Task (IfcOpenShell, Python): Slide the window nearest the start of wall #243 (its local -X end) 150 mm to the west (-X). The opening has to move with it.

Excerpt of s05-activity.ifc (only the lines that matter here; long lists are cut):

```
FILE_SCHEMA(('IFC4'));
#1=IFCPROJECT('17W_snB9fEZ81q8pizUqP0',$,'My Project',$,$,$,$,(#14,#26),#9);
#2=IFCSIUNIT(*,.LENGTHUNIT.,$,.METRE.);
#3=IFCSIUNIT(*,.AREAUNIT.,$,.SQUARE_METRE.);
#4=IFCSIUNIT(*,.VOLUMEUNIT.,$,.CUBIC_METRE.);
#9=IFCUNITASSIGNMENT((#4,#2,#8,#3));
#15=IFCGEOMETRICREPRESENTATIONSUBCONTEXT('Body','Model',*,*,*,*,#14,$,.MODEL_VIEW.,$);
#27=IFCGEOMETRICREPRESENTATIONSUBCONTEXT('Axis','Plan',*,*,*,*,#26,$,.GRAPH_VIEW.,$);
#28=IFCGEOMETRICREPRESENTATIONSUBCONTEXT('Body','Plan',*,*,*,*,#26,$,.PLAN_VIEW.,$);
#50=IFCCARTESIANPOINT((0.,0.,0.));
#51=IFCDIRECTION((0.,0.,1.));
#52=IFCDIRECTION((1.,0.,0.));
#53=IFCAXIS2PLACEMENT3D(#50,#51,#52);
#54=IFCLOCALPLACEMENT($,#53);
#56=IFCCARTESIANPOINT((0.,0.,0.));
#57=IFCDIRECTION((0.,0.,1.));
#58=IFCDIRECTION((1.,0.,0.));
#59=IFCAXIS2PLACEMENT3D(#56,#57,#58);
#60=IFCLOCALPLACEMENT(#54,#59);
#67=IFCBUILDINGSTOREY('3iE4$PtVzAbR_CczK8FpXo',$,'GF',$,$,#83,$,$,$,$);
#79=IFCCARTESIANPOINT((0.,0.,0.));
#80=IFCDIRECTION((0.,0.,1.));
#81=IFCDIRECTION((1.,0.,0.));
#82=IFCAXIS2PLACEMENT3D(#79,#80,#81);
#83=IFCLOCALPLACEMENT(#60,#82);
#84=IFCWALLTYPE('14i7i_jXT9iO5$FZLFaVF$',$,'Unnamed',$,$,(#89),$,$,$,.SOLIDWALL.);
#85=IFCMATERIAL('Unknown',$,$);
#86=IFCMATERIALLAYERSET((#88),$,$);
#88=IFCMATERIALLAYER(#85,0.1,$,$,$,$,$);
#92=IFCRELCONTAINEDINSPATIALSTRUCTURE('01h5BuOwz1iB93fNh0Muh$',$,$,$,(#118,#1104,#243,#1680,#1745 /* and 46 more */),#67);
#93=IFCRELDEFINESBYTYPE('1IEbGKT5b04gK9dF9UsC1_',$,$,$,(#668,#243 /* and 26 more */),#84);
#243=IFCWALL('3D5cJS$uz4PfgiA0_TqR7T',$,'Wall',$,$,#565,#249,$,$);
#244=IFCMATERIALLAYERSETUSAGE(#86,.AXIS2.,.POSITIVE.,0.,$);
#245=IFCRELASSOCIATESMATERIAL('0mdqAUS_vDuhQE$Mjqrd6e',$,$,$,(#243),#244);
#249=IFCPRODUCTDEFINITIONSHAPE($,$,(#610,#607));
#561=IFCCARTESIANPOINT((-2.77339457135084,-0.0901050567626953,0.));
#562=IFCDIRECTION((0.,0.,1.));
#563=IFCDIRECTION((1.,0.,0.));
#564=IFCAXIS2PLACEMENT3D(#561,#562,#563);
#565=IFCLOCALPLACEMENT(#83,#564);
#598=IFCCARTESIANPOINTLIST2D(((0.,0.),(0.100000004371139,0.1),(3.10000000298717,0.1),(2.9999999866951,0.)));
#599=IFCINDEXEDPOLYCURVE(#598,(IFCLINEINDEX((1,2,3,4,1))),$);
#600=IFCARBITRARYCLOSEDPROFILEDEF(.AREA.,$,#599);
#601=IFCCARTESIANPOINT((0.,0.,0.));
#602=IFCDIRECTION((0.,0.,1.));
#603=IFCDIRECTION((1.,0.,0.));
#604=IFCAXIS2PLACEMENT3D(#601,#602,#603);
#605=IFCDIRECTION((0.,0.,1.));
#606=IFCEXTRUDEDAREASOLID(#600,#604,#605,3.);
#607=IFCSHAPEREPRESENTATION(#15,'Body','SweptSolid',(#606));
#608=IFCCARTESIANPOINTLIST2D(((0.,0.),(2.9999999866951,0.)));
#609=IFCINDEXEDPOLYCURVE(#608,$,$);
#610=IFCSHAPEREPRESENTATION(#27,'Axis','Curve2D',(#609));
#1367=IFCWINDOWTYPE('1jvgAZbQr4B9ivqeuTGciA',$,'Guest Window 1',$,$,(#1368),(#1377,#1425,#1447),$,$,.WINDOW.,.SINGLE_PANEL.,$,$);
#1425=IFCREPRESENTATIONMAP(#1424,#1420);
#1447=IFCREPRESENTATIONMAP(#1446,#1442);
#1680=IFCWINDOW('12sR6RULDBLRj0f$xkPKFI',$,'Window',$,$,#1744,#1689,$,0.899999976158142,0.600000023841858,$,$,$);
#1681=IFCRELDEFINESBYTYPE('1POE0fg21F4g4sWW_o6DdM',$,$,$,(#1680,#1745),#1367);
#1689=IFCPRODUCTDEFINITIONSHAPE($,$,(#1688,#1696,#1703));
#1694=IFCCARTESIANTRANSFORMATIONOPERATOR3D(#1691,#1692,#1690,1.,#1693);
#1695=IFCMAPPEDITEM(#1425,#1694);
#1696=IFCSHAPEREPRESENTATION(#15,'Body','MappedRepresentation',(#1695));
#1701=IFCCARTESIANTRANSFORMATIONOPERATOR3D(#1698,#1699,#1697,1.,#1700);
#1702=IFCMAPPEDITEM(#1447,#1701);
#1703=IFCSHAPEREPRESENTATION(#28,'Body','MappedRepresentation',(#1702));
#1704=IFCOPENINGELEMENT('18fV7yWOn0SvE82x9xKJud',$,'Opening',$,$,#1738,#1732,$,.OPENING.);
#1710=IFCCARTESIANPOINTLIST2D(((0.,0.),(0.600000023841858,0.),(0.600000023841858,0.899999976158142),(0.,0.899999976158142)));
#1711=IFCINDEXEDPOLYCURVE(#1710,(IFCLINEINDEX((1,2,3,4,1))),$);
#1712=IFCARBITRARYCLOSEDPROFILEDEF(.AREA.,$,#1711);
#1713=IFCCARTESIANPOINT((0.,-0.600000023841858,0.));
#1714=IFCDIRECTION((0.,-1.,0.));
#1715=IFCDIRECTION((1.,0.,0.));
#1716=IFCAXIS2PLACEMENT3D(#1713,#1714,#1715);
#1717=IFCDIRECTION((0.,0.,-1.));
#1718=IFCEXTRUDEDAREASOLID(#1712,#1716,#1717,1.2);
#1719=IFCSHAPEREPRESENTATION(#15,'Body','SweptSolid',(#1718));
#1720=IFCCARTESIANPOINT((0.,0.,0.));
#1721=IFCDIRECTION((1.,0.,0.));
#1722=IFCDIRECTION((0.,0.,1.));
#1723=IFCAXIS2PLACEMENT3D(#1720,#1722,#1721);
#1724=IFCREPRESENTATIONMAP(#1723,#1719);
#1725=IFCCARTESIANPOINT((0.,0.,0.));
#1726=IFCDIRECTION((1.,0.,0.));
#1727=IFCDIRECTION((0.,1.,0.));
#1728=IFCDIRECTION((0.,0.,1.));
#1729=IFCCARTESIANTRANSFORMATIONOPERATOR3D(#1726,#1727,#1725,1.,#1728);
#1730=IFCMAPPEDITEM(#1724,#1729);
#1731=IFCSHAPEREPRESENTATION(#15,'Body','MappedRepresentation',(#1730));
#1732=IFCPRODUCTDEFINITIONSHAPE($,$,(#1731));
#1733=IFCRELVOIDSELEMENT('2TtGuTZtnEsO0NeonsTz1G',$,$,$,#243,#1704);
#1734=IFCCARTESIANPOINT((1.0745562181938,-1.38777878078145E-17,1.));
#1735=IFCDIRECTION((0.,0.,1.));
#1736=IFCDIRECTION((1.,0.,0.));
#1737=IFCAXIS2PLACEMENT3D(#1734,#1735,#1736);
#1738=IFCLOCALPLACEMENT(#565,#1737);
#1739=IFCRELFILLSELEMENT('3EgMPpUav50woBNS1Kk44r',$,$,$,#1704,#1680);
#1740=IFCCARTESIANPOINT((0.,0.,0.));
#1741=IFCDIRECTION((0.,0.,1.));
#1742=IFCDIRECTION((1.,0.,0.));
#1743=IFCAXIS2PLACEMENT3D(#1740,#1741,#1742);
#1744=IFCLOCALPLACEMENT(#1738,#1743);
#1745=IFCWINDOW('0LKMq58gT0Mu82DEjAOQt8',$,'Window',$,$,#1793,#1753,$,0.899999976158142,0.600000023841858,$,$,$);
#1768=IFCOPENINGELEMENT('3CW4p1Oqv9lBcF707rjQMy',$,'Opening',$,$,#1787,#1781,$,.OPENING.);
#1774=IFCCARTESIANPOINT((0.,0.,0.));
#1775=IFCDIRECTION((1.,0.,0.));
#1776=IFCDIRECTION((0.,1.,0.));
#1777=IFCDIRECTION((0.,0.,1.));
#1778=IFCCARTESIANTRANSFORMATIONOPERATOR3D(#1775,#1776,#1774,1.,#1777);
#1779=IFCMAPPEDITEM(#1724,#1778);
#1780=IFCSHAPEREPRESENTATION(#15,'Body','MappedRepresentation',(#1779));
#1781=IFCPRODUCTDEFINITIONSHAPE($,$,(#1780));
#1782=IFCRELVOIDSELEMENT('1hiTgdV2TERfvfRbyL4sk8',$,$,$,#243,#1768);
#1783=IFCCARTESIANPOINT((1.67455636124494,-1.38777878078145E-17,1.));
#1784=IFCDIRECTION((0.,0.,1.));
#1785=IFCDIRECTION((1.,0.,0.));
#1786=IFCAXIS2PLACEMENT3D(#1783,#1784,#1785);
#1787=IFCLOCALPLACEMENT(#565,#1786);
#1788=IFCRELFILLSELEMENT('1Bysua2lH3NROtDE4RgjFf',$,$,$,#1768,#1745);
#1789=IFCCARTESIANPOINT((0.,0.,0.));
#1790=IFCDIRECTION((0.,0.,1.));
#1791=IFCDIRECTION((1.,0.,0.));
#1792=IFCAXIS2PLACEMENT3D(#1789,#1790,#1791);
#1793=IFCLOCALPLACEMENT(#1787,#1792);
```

```python
import ifcopenshell
import ifcopenshell.api.geometry
import ifcopenshell.util.placement
import ifcopenshell.util.unit

model = ifcopenshell.open("s05-activity.ifc")
unit_scale = ifcopenshell.util.unit.calculate_unit_scale(model)

window = model.by_guid("12sR6RULDBLRj0f$xkPKFI")
opening = window.FillsVoids[0].RelatingOpeningElement
wall = opening.VoidsElements[0].RelatingBuildingElement

wall_matrix = ifcopenshell.util.placement.get_local_placement(wall.ObjectPlacement)
shift = wall_matrix[:3, 0] * -0.15 / unit_scale
before = ifcopenshell.util.placement.get_local_placement(window.ObjectPlacement)[:3, 3].copy()

# The window is placed relative to its opening, so it follows when the opening moves.
matrix = ifcopenshell.util.placement.get_local_placement(opening.ObjectPlacement)
matrix[:3, 3] += shift
ifcopenshell.api.geometry.edit_object_placement(
    model, product=opening, matrix=matrix, is_si=False, should_transform_children=True
)

after = ifcopenshell.util.placement.get_local_placement(window.ObjectPlacement)[:3, 3]
print("window moved by", (after - before).round(3) + 0.0)

model.write("s05-activity_edited.ifc")
```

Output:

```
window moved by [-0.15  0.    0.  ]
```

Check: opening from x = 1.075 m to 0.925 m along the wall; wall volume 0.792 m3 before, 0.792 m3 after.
